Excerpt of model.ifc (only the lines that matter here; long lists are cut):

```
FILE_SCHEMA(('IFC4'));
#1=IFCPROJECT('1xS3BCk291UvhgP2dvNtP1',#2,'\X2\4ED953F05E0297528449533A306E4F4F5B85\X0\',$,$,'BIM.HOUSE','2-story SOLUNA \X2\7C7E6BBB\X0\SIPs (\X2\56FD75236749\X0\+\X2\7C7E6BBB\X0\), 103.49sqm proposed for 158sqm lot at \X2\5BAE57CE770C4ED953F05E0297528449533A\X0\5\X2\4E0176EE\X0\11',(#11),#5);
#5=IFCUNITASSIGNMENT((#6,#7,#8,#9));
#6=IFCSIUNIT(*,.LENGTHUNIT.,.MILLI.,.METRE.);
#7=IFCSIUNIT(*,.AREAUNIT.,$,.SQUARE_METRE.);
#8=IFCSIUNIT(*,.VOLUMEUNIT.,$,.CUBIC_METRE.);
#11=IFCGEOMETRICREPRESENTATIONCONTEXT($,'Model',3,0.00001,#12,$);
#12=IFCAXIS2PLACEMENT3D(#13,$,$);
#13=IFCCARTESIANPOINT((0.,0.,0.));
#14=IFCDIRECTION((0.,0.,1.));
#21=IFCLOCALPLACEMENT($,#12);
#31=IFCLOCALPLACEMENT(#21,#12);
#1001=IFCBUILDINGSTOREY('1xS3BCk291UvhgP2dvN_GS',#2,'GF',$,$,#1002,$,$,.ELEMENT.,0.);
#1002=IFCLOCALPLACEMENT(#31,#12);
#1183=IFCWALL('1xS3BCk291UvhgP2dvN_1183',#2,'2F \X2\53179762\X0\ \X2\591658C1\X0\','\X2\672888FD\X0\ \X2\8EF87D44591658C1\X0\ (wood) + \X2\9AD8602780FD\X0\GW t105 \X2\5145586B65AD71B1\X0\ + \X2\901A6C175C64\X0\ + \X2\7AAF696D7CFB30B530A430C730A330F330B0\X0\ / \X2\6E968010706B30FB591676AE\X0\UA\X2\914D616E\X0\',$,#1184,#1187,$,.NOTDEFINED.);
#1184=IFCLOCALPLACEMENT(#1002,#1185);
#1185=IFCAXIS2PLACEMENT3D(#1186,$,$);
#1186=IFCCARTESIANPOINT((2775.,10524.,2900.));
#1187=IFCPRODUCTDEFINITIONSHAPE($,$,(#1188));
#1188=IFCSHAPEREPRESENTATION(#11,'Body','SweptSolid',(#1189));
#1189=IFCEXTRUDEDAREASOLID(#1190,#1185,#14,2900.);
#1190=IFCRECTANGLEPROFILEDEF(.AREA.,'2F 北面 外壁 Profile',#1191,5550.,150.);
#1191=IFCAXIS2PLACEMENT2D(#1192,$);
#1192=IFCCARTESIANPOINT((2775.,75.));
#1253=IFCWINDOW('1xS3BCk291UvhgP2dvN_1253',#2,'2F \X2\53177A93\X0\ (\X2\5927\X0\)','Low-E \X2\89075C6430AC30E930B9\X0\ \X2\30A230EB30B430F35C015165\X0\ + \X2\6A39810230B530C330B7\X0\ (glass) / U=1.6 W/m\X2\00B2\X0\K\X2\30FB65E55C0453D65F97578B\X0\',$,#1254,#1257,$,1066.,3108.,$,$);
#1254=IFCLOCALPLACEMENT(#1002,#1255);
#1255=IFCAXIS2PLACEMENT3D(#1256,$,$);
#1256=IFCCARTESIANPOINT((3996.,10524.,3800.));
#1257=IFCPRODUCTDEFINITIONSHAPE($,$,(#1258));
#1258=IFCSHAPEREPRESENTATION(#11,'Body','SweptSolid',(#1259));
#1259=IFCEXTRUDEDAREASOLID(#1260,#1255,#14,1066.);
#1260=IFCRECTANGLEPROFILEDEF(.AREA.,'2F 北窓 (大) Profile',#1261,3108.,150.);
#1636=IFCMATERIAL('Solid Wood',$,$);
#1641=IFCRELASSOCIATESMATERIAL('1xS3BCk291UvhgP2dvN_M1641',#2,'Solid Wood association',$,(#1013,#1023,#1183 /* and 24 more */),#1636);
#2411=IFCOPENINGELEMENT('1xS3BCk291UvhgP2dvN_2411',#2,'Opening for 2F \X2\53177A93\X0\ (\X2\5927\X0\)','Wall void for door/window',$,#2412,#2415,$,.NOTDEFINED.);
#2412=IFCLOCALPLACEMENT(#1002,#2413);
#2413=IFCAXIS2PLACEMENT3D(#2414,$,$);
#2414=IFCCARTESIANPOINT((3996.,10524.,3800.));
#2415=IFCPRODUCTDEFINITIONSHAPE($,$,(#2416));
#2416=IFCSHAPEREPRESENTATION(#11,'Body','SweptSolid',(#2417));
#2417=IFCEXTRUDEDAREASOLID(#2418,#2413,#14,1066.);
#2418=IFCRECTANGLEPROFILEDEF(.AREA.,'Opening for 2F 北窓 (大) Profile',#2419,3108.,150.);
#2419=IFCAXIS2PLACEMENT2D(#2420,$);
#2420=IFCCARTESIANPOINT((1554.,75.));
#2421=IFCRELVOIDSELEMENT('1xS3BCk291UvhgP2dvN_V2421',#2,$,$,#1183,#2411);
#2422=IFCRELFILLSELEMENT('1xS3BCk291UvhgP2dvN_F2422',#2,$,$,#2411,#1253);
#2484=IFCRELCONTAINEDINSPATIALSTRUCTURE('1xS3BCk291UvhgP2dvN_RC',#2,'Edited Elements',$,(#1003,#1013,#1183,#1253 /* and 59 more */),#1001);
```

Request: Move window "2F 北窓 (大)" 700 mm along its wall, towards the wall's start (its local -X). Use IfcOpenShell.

```python
import ifcopenshell
import ifcopenshell.api.geometry
import ifcopenshell.util.placement

model = ifcopenshell.open("model.ifc")

window = model.by_guid("1xS3BCk291UvhgP2dvN_1253")
opening = window.FillsVoids[0].RelatingOpeningElement
wall = opening.VoidsElements[0].RelatingBuildingElement

wall_matrix = ifcopenshell.util.placement.get_local_placement(wall.ObjectPlacement)
shift = wall_matrix[:3, 0] * -700.0
before = ifcopenshell.util.placement.get_local_placement(window.ObjectPlacement)[:3, 3].copy()

# The window is not placed relative to its opening, so move both.
for product in (opening, window):
    matrix = ifcopenshell.util.placement.get_local_placement(product.ObjectPlacement)
    matrix[:3, 3] += shift
    ifcopenshell.api.geometry.edit_object_placement(model, product=product, matrix=matrix, is_si=False)

after = ifcopenshell.util.placement.get_local_placement(window.ObjectPlacement)[:3, 3]
print("window moved by", (after - before).round(3) + 0.0)

model.write("model-out.ifc")
```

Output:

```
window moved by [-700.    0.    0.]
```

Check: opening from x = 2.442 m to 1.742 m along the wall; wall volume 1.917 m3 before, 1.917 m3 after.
